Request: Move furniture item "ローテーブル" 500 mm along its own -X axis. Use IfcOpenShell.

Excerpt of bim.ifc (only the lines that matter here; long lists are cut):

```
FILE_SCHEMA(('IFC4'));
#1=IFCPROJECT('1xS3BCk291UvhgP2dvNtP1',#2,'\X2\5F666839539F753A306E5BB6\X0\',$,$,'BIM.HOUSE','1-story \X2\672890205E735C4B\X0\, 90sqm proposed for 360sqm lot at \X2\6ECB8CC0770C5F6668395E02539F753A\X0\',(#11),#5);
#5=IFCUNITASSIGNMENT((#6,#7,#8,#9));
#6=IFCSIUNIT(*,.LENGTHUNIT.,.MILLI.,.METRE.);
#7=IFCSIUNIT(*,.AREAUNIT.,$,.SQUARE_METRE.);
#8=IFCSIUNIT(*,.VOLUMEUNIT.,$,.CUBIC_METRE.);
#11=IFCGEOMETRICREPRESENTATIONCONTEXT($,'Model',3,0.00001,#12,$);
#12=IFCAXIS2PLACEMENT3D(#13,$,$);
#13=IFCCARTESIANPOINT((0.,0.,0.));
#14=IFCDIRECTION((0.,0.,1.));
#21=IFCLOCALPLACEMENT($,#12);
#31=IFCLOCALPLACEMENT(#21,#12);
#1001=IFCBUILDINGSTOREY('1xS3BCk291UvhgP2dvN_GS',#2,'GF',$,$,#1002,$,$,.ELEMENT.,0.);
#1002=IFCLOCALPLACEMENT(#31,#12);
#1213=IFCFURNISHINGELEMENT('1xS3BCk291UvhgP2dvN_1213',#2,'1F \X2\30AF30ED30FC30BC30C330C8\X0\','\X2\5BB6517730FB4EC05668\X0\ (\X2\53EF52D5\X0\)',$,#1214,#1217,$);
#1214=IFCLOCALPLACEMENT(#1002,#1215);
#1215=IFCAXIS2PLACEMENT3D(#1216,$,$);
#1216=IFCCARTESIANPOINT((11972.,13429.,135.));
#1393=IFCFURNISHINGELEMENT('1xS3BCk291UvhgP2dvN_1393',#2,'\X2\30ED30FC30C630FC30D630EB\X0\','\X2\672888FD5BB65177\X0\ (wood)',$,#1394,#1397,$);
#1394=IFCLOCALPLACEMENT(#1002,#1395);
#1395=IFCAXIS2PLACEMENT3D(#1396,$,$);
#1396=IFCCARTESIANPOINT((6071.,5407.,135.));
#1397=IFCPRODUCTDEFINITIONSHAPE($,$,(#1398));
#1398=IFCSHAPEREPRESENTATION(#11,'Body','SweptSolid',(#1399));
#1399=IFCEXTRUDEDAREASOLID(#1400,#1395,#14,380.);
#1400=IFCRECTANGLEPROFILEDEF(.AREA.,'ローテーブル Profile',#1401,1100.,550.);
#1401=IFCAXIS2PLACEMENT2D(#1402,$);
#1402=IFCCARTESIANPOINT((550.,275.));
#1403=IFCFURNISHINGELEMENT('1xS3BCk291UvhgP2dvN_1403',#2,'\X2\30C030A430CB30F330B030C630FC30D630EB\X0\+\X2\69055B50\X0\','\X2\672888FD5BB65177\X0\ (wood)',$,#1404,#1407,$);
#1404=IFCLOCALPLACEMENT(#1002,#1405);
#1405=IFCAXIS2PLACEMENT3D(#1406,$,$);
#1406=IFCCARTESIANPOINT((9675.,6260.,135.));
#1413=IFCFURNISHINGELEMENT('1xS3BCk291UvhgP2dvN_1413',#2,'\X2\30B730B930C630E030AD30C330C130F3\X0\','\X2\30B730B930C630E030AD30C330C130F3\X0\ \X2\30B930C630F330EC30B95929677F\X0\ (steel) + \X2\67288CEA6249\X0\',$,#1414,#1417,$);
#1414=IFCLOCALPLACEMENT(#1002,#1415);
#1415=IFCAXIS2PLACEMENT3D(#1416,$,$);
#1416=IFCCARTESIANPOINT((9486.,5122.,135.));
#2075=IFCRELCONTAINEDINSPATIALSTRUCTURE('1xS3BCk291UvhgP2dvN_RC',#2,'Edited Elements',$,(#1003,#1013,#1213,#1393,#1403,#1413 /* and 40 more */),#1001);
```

```python
import ifcopenshell
import ifcopenshell.api.geometry
import ifcopenshell.util.placement
import ifcopenshell.util.unit

model = ifcopenshell.open("bim.ifc")
unit_scale = ifcopenshell.util.unit.calculate_unit_scale(model)

item = model.by_id(1393)
matrix = ifcopenshell.util.placement.get_local_placement(item.ObjectPlacement)
matrix[:3, 3] -= matrix[:3, 0] * 0.5 / unit_scale
ifcopenshell.api.geometry.edit_object_placement(model, product=item, matrix=matrix, is_si=False)

print(ifcopenshell.util.placement.get_local_placement(item.ObjectPlacement).round(3) + 0.0)

model.write("bim_v2.ifc")
```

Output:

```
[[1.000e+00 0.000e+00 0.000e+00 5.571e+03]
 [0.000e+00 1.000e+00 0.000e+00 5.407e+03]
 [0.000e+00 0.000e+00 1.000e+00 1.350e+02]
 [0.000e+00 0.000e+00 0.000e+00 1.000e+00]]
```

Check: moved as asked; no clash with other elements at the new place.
